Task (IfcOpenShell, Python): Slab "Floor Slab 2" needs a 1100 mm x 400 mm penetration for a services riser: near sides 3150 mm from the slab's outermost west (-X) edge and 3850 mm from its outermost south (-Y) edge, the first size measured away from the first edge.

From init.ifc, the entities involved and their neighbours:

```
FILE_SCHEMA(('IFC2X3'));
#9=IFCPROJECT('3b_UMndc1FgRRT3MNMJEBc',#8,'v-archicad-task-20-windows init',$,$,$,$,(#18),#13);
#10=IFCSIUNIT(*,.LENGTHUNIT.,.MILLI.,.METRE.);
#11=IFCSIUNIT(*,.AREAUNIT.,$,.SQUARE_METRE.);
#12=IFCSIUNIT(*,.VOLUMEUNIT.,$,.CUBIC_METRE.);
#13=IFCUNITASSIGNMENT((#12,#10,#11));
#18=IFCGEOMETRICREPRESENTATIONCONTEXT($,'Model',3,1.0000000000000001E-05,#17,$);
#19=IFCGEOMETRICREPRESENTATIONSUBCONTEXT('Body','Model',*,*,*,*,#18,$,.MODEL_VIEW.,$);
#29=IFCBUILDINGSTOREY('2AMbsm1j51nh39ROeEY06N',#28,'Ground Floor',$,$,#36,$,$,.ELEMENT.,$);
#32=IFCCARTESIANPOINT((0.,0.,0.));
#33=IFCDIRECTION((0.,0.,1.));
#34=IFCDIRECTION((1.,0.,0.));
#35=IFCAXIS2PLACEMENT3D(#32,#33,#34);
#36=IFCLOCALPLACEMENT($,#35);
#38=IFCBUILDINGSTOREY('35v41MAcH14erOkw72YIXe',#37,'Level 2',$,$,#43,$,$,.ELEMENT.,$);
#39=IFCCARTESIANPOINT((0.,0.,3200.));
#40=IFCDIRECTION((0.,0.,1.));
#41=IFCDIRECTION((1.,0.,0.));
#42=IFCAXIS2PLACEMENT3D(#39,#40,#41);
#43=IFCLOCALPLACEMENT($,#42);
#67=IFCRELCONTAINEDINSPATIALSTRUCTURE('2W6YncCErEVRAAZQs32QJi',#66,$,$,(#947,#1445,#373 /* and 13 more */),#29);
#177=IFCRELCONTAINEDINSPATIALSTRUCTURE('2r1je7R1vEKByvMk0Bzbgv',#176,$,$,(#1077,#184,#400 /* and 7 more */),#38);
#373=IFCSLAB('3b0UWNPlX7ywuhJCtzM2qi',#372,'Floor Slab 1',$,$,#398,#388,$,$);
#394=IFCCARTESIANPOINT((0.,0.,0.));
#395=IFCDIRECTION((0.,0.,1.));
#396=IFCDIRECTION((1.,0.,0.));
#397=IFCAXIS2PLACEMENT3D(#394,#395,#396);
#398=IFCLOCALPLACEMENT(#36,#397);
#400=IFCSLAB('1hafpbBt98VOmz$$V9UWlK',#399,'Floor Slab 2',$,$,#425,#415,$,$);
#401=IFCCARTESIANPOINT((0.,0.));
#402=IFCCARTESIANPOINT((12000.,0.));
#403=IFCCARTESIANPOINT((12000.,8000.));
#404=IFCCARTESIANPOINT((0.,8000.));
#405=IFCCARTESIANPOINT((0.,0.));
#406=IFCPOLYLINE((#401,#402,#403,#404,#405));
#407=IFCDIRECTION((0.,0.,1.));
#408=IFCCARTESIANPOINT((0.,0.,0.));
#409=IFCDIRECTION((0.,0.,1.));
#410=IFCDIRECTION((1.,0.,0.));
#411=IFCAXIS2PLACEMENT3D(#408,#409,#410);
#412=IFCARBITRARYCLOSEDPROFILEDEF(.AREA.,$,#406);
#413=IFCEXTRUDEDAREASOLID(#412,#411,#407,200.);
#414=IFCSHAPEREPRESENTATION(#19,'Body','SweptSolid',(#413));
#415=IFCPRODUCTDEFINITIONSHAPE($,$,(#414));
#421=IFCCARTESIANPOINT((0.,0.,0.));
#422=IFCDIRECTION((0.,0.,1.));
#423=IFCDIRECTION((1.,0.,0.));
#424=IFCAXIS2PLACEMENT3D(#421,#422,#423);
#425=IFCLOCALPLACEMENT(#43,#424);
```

```python
import numpy as np
import ifcopenshell
import ifcopenshell.api.feature
import ifcopenshell.api.geometry
import ifcopenshell.api.root
import ifcopenshell.geom
import ifcopenshell.util.placement
import ifcopenshell.util.representation
import ifcopenshell.util.shape
import ifcopenshell.util.unit

model = ifcopenshell.open("init.ifc")
unit_scale = ifcopenshell.util.unit.calculate_unit_scale(model)
settings = ifcopenshell.geom.settings()


def volume(element):
    """Net volume in cubic metres, openings subtracted."""
    shape = ifcopenshell.geom.create_shape(settings, element)
    return ifcopenshell.util.shape.get_volume(shape.geometry)


slab = model.by_id(400)
before = volume(slab)

# Extent in the slab's own axes, in metres. The edges named are its -X and -Y sides.
slab_shape = ifcopenshell.geom.create_shape(settings, slab)
vertices = ifcopenshell.util.shape.get_vertices(slab_shape.geometry)
x_min, y_min, bottom = vertices.min(axis=0)
top = vertices[:, 2].max()

opening = ifcopenshell.api.root.create_entity(model, ifc_class="IfcOpeningElement", name="Services riser opening")
context = ifcopenshell.util.representation.get_context(model, "Model", "Body", "MODEL_VIEW")
width, depth = 1.1, 0.4
outline = [(0.0, 0.0), (width, 0.0), (width, depth), (0.0, depth), (0.0, 0.0)]
# Overshoot both faces by 50 mm so the cut is clean.
shape = ifcopenshell.api.geometry.add_slab_representation(
    model, context=context, depth=top - bottom + 0.1, polyline=outline
)
ifcopenshell.api.geometry.assign_representation(model, product=opening, representation=shape)

matrix = ifcopenshell.util.placement.get_local_placement(slab.ObjectPlacement)
matrix[:, 3] = matrix @ np.append(np.array([x_min + 3.15, y_min + 3.85, bottom - 0.05]) / unit_scale, 1.0)
ifcopenshell.api.geometry.edit_object_placement(model, product=opening, matrix=matrix, is_si=False)
ifcopenshell.api.feature.add_feature(model, feature=opening, element=slab)

after = volume(slab)

print(f"slab volume {before:.3f} -> {after:.3f} m3")

model.write("init_updated.ifc")
```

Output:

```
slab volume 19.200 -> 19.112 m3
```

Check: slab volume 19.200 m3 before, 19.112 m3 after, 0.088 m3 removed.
